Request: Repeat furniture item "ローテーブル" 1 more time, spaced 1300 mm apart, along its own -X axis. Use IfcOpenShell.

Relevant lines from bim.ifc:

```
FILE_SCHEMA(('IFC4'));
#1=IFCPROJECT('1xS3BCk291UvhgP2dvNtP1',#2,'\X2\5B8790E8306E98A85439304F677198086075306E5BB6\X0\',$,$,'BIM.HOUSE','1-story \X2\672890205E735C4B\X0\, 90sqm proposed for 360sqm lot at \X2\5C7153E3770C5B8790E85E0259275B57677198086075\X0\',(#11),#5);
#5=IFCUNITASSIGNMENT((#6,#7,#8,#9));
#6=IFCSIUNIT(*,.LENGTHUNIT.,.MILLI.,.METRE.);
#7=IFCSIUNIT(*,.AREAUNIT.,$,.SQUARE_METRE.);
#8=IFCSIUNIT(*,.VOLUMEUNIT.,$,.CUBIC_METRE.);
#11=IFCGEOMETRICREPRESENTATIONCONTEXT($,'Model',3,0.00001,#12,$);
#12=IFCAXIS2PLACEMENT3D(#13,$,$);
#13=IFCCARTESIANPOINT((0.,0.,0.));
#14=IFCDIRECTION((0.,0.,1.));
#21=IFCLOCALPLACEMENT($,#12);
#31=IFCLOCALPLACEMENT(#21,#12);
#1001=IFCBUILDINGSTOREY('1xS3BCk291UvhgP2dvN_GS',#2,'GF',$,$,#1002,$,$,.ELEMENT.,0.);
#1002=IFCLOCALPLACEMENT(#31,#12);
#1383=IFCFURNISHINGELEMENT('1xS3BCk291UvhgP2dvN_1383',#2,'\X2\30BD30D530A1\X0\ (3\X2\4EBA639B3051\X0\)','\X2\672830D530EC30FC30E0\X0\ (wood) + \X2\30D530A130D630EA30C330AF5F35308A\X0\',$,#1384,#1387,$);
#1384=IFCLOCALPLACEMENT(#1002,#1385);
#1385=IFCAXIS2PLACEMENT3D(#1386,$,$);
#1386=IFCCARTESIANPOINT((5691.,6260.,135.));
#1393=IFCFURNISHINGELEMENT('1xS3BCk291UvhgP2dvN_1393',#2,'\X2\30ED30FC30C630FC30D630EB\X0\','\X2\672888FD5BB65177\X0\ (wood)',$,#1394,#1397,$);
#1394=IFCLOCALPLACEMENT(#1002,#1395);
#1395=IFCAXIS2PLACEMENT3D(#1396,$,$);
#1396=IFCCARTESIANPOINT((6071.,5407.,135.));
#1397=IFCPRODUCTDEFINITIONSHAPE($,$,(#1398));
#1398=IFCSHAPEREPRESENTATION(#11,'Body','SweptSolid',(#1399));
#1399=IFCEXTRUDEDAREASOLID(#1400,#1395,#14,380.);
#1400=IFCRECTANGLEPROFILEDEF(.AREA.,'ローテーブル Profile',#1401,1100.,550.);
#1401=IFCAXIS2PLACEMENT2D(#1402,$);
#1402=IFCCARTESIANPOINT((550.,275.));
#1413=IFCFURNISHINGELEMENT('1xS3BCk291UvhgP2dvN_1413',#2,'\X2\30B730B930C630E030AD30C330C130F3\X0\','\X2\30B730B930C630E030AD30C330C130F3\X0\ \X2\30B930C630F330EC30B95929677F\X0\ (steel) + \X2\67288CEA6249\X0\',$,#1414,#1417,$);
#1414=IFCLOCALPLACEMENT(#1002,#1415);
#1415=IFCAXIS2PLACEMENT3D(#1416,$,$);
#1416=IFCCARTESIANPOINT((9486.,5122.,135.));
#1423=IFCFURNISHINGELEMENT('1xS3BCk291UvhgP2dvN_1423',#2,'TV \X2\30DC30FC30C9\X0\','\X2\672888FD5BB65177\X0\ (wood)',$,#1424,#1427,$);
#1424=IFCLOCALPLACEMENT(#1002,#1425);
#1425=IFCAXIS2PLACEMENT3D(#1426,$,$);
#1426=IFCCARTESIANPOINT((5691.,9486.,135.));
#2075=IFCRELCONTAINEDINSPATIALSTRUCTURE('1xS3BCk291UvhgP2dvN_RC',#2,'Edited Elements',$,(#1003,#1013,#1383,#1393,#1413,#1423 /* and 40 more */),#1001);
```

```python
import ifcopenshell
import ifcopenshell.api.geometry
import ifcopenshell.api.root
import ifcopenshell.util.element
import ifcopenshell.util.placement
import ifcopenshell.util.unit

model = ifcopenshell.open("bim.ifc")
unit_scale = ifcopenshell.util.unit.calculate_unit_scale(model)


def reuse_history(source, copy):
    """copy_class also copies each property set's owner history, people and application; keep the originals."""
    for rel in copy.IsDefinedBy:
        if rel.is_a("IfcRelDefinesByProperties") and (history := rel.RelatingPropertyDefinition.OwnerHistory):
            rel.RelatingPropertyDefinition.OwnerHistory = source.OwnerHistory
            ifcopenshell.util.element.remove_deep2(model, history)


source = model.by_id(1393)
base = ifcopenshell.util.placement.get_local_placement(source.ObjectPlacement)
step = -base[:3, 0] * 1.3 / unit_scale

for i in range(1, 2):
    copy = ifcopenshell.api.root.copy_class(model, product=source)
    copy.Representation = ifcopenshell.util.element.copy_deep(
        model, source.Representation, exclude=["IfcGeometricRepresentationContext", "IfcRepresentationMap"]
    )
    reuse_history(source, copy)
    matrix = base.copy()
    matrix[:3, 3] += i * step
    print("added at", matrix[:3, 3].round(3) + 0.0)
    ifcopenshell.api.geometry.edit_object_placement(model, product=copy, matrix=matrix, is_si=False)

model.write("bim_rev.ifc")
```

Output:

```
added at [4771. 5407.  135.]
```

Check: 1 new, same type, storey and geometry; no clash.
